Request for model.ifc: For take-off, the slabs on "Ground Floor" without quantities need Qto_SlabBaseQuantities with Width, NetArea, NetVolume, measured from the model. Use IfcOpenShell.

First a look at what the model holds.

```python
import ifcopenshell
import ifcopenshell.util.element
import ifcopenshell.util.unit

model = ifcopenshell.open("model.ifc")
print(model.schema)
for unit_type in ("LENGTHUNIT", "AREAUNIT", "VOLUMEUNIT"):
    print(unit_type, ifcopenshell.util.unit.calculate_unit_scale(model, unit_type))
storey = next(s for s in model.by_type("IfcBuildingStorey") if s.Name == "Ground Floor")
slabs = [e for e in ifcopenshell.util.element.get_decomposition(storey) if e.is_a("IfcSlab")]
for e in sorted(slabs, key=lambda e: e.id()):
    print(e.id(), e.is_a(), e.Name, list(ifcopenshell.util.element.get_psets(e, qtos_only=True)), sep=" | ")
```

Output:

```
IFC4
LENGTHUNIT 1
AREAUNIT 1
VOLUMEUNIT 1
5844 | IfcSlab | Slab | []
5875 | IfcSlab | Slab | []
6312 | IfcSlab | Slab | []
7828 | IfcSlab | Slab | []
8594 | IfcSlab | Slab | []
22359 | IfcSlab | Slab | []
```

```python
import ifcopenshell
import ifcopenshell.api.pset
import ifcopenshell.geom
import ifcopenshell.util.element
import ifcopenshell.util.shape
import ifcopenshell.util.unit

model = ifcopenshell.open("model.ifc")
unit_scale = ifcopenshell.util.unit.calculate_unit_scale(model)
area_scale = ifcopenshell.util.unit.calculate_unit_scale(model, "AREAUNIT")
volume_scale = ifcopenshell.util.unit.calculate_unit_scale(model, "VOLUMEUNIT")
settings = ifcopenshell.geom.settings()

storey = next(s for s in model.by_type("IfcBuildingStorey") if s.Name == "Ground Floor")
slabs = [e for e in ifcopenshell.util.element.get_decomposition(storey) if e.is_a("IfcSlab")]

for e in sorted(slabs, key=lambda e: e.id()):
    if ifcopenshell.util.element.get_psets(e, qtos_only=True, should_inherit=False):
        continue
    # Geometry comes back in metres, in the element's own axes.
    shape = ifcopenshell.geom.create_shape(settings, e)
    values = {
        "Width": ifcopenshell.util.shape.get_z(shape.geometry) / unit_scale,
        "NetArea": ifcopenshell.util.shape.get_footprint_area(shape.geometry) / area_scale,
        "NetVolume": ifcopenshell.util.shape.get_volume(shape.geometry) / volume_scale,
    }
    qto = ifcopenshell.api.pset.add_qto(model, product=e, name="Qto_SlabBaseQuantities")
    ifcopenshell.api.pset.edit_qto(model, qto=qto, properties=values)
    print(e.id(), {k: round(v, 3) for k, v in values.items()})

model.write("model_v2.ifc")
```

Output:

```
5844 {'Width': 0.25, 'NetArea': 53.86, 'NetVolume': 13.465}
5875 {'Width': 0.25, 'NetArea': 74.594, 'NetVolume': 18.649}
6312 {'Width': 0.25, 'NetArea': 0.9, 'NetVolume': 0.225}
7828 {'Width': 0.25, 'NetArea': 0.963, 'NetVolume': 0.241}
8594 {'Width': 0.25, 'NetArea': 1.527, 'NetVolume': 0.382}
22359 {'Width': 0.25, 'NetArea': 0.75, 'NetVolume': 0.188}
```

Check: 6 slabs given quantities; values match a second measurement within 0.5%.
